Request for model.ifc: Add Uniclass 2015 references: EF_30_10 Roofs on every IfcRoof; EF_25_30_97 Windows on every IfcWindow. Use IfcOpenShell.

First a look at what the model holds.

```python
import ifcopenshell

model = ifcopenshell.open("model.ifc")
print(model.schema)
print("classifications:", [c.Name for c in model.by_type("IfcClassification")])
for ifc_class in ("IfcDoor", "IfcRoof", "IfcStair", "IfcWall", "IfcWindow"):
    print(ifc_class, len(model.by_type(ifc_class)))
```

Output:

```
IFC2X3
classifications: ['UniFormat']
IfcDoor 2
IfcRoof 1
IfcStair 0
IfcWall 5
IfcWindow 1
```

```python
import ifcopenshell
import ifcopenshell.api.classification

model = ifcopenshell.open("model.ifc")

# IFC2X3 requires Source and Edition and has no link from the project to the system.
system = model.create_entity("IfcClassification", Source="NBS", Edition="2015", Name="Uniclass 2015")

codes = {
    "IfcRoof": ("EF_30_10", "Roofs"),
    "IfcWindow": ("EF_25_30_97", "Windows"),
}
for ifc_class, (code, name) in codes.items():
    products = model.by_type(ifc_class)
    ifcopenshell.api.classification.add_reference(
        model, products=products, classification=system, identification=code, name=name
    )
    print(code, len(products))

model.write("model_v2.ifc")
```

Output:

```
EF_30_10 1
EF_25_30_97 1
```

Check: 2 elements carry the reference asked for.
